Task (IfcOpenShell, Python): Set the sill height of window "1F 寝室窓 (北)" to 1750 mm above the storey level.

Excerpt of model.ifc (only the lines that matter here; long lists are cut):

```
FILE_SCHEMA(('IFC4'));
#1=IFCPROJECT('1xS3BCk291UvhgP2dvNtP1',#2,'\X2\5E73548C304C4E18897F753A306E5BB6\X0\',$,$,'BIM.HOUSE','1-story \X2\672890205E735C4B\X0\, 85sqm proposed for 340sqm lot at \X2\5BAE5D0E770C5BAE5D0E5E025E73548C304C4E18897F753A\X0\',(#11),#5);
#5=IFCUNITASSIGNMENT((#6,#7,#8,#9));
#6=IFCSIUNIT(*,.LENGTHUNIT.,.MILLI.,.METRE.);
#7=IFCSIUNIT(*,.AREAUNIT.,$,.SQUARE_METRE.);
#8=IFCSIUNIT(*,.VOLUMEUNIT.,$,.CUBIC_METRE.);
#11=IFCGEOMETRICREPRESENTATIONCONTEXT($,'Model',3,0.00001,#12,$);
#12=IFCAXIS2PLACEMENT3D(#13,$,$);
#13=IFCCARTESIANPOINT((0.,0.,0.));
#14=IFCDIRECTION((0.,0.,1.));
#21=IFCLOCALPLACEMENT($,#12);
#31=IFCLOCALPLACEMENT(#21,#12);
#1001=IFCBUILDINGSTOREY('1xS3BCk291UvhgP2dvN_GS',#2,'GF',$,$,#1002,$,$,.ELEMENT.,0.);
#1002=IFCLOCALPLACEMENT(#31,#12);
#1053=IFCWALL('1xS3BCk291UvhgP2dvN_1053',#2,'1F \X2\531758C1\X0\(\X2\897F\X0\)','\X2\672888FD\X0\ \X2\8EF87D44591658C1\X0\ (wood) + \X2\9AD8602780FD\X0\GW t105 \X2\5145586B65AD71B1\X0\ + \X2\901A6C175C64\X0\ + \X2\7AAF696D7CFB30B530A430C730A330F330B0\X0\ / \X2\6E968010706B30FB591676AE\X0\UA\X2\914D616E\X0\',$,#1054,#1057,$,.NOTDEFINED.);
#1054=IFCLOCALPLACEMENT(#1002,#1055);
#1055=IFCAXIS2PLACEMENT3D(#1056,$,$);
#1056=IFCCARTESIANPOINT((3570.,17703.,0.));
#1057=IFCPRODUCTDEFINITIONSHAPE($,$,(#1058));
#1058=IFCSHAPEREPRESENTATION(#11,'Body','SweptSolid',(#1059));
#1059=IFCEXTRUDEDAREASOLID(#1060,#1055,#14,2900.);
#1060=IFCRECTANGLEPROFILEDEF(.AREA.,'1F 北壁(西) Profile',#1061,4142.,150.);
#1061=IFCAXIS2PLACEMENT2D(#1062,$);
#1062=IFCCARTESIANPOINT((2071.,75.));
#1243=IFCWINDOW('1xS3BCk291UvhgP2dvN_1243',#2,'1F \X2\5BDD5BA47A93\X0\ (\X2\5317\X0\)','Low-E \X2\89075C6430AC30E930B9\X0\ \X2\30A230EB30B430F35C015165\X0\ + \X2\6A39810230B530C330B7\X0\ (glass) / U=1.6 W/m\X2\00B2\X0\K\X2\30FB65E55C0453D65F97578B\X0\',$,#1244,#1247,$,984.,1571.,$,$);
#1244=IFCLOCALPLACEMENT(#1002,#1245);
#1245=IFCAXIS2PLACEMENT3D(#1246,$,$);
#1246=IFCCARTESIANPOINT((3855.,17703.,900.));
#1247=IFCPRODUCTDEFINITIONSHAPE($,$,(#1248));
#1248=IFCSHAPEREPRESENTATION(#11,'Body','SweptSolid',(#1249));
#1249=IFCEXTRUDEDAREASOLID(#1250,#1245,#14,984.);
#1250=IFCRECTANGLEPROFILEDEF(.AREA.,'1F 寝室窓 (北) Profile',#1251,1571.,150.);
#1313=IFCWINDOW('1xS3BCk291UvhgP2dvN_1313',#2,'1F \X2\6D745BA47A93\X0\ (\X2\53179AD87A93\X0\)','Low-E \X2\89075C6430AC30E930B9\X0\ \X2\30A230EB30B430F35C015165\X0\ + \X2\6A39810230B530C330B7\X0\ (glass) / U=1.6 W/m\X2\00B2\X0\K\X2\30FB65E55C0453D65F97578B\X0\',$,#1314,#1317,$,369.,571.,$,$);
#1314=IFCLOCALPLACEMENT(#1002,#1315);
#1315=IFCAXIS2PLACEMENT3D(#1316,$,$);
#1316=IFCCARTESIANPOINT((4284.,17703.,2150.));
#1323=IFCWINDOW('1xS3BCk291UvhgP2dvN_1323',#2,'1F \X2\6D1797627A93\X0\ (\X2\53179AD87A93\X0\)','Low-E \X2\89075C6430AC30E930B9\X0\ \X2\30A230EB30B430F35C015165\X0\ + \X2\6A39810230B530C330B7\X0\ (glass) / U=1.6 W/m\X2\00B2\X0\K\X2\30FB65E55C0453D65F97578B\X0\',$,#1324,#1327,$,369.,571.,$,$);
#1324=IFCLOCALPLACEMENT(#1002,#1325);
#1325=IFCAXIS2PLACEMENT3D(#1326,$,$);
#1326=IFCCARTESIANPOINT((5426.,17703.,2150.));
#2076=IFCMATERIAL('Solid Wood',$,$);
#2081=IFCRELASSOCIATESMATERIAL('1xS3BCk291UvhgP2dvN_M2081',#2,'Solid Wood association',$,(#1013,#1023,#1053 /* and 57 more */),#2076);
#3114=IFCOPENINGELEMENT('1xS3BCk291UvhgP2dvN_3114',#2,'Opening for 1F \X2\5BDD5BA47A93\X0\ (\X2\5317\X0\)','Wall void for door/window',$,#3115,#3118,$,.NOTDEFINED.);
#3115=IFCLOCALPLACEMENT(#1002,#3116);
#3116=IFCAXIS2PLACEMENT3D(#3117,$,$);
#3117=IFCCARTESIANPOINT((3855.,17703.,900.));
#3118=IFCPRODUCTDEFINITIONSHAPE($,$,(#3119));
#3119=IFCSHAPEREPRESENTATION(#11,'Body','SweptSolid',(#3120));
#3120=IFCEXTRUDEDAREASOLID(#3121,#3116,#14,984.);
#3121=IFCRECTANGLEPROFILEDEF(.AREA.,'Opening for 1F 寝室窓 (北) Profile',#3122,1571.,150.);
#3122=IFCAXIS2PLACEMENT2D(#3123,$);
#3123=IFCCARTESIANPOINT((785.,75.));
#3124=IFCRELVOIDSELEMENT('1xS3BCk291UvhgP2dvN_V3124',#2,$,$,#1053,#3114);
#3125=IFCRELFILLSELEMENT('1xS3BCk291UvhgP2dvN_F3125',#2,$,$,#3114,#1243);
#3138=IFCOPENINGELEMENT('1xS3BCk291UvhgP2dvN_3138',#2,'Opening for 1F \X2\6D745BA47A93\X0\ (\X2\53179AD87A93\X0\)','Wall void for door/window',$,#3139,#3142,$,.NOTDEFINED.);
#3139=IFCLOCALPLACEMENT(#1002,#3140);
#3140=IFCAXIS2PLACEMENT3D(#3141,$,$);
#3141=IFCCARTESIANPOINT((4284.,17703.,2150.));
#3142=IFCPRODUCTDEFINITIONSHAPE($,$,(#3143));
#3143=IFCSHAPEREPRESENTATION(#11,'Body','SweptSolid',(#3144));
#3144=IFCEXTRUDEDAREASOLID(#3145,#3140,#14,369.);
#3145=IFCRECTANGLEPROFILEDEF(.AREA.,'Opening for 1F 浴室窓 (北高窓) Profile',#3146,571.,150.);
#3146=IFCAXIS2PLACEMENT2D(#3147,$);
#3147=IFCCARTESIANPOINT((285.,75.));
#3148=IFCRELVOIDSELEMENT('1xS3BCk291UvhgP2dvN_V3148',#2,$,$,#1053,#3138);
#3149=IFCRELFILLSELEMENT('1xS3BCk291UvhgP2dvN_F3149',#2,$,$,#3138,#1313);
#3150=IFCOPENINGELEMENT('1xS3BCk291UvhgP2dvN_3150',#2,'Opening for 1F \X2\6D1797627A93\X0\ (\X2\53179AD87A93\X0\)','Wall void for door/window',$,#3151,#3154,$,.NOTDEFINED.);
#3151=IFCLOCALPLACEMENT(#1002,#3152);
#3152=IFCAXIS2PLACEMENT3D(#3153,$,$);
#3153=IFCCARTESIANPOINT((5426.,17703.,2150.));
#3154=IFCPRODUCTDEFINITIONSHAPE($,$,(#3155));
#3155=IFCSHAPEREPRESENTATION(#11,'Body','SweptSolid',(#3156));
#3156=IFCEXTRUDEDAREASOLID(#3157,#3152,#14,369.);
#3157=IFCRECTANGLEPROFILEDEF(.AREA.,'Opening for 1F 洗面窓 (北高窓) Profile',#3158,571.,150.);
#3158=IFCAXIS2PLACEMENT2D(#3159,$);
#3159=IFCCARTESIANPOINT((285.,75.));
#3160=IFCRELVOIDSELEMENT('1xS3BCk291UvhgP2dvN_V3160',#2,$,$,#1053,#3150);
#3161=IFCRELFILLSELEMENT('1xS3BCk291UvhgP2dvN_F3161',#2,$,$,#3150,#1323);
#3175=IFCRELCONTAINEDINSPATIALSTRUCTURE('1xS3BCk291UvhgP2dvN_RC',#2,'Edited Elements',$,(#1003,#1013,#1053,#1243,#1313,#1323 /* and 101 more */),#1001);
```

```python
import numpy as np
import ifcopenshell
import ifcopenshell.api.geometry
import ifcopenshell.geom
import ifcopenshell.util.element
import ifcopenshell.util.placement
import ifcopenshell.util.shape
import ifcopenshell.util.unit

model = ifcopenshell.open("model.ifc")
unit_scale = ifcopenshell.util.unit.calculate_unit_scale(model)

window = model.by_id(1243)
opening = window.FillsVoids[0].RelatingOpeningElement
storey = ifcopenshell.util.element.get_container(window, ifc_class="IfcBuildingStorey")
level = ifcopenshell.util.placement.get_local_placement(storey.ObjectPlacement)[2, 3]

# The opening's origin need not be at the sill, so measure its lowest point.
shape = ifcopenshell.geom.create_shape(ifcopenshell.geom.settings(), opening)
bottom = ifcopenshell.util.shape.get_shape_bottom_elevation(shape, shape.geometry) / unit_scale
dz = level + 1.75 / unit_scale - bottom

shift = np.array([0.0, 0.0, dz])
# The window is not placed relative to its opening, so move both.
for product in (opening, window):
    matrix = ifcopenshell.util.placement.get_local_placement(product.ObjectPlacement)
    matrix[:3, 3] += shift
    ifcopenshell.api.geometry.edit_object_placement(model, product=product, matrix=matrix, is_si=False)

print(f"moved by {dz * unit_scale:+.3f} m")

model.write("model-out.ifc")
```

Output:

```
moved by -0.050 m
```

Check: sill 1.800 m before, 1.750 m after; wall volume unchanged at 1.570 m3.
